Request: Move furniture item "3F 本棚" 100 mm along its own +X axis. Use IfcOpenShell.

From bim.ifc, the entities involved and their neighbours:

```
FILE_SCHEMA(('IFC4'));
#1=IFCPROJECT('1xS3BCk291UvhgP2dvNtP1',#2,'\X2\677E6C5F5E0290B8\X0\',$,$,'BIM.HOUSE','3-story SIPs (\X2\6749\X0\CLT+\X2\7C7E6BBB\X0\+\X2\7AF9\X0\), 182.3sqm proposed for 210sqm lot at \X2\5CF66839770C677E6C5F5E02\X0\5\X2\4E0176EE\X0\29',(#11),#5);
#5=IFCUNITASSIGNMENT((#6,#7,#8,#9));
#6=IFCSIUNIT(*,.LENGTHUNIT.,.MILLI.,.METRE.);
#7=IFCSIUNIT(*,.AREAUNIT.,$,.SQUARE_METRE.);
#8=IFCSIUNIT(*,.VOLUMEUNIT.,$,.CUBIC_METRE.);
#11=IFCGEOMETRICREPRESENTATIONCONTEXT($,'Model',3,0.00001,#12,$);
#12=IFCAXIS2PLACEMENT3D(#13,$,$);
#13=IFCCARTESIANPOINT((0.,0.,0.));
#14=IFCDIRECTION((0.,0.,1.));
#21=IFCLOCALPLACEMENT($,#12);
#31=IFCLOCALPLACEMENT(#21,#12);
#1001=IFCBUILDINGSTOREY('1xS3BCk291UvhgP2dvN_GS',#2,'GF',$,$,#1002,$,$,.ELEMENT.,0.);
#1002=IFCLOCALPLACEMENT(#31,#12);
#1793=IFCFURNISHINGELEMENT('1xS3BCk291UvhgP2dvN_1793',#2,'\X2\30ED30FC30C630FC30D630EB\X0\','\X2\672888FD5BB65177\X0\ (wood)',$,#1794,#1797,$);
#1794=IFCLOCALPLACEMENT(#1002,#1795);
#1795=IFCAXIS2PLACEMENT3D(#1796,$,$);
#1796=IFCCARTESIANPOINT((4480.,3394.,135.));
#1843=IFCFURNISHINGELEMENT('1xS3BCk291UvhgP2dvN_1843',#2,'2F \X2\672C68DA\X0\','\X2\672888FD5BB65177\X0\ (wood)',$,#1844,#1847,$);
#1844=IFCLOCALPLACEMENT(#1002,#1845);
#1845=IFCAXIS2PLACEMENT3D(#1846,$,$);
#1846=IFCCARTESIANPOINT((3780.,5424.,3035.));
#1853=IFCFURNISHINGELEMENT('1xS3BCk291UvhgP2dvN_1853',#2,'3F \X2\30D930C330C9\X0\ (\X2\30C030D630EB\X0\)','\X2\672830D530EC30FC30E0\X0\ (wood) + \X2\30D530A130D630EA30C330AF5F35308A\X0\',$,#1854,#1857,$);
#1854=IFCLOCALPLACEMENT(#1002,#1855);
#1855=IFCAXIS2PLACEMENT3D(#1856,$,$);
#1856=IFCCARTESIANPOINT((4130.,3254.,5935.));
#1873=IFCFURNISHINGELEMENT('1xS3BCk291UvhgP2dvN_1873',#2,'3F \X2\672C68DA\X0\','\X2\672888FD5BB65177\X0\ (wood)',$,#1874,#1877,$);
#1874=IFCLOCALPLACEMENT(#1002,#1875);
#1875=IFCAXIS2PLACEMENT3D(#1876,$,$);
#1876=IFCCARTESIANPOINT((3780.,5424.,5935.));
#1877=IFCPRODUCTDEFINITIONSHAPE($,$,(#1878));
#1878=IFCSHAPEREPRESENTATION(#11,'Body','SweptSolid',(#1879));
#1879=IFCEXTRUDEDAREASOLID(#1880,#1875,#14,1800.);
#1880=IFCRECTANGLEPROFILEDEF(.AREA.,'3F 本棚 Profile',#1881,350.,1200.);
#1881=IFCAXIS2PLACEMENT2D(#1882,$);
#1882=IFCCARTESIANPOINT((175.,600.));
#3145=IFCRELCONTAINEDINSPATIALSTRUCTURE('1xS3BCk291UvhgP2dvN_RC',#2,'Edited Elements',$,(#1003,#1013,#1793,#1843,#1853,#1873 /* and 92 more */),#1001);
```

```python
import ifcopenshell
import ifcopenshell.api.geometry
import ifcopenshell.util.placement

model = ifcopenshell.open("bim.ifc")

item = model.by_guid("1xS3BCk291UvhgP2dvN_1873")
matrix = ifcopenshell.util.placement.get_local_placement(item.ObjectPlacement)
matrix[:3, 3] += matrix[:3, 0] * 100.0
ifcopenshell.api.geometry.edit_object_placement(model, product=item, matrix=matrix, is_si=False)

print(ifcopenshell.util.placement.get_local_placement(item.ObjectPlacement).round(3) + 0.0)

model.write("bim-out.ifc")
```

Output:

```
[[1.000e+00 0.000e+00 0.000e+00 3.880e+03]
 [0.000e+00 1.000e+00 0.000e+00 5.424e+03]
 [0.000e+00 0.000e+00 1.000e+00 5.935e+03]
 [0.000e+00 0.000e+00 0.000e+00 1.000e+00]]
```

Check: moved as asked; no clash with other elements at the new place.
